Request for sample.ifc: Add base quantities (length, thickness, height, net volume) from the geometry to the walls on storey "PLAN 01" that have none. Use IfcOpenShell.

First a look at what the model holds.

```python
import ifcopenshell
import ifcopenshell.util.element
import ifcopenshell.util.unit

model = ifcopenshell.open("sample.ifc")
print(model.schema)
for unit_type in ("LENGTHUNIT", "AREAUNIT", "VOLUMEUNIT"):
    print(unit_type, ifcopenshell.util.unit.calculate_unit_scale(model, unit_type))
storey = next(s for s in model.by_type("IfcBuildingStorey") if s.Name == "PLAN 01")
walls = [e for e in ifcopenshell.util.element.get_decomposition(storey) if e.is_a("IfcWall")]
for e in sorted(walls, key=lambda e: e.id()):
    print(e.id(), e.is_a(), e.Name, list(ifcopenshell.util.element.get_psets(e, qtos_only=True)), sep=" | ")
```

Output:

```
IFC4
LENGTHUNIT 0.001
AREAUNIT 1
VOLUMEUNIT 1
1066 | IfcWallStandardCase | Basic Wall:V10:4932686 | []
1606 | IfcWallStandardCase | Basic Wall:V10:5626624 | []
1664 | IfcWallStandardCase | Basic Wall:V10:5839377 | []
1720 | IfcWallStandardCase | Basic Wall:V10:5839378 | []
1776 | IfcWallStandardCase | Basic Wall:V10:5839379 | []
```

```python
import ifcopenshell
import ifcopenshell.api.pset
import ifcopenshell.geom
import ifcopenshell.util.element
import ifcopenshell.util.shape
import ifcopenshell.util.unit

model = ifcopenshell.open("sample.ifc")
unit_scale = ifcopenshell.util.unit.calculate_unit_scale(model)
volume_scale = ifcopenshell.util.unit.calculate_unit_scale(model, "VOLUMEUNIT")
settings = ifcopenshell.geom.settings()

storey = next(s for s in model.by_type("IfcBuildingStorey") if s.Name == "PLAN 01")
walls = [e for e in ifcopenshell.util.element.get_decomposition(storey) if e.is_a("IfcWall")]

for e in sorted(walls, key=lambda e: e.id()):
    if ifcopenshell.util.element.get_psets(e, qtos_only=True, should_inherit=False):
        continue
    # Geometry comes back in metres, in the element's own axes.
    shape = ifcopenshell.geom.create_shape(settings, e)
    values = {
        "Length": ifcopenshell.util.shape.get_x(shape.geometry) / unit_scale,
        "Width": ifcopenshell.util.shape.get_y(shape.geometry) / unit_scale,
        "Height": ifcopenshell.util.shape.get_z(shape.geometry) / unit_scale,
        "NetVolume": ifcopenshell.util.shape.get_volume(shape.geometry) / volume_scale,
    }
    qto = ifcopenshell.api.pset.add_qto(model, product=e, name="Qto_WallBaseQuantities")
    ifcopenshell.api.pset.edit_qto(model, qto=qto, properties=values)
    print(e.id(), {k: round(v, 3) for k, v in values.items()})

model.write("sample_edited.ifc")
```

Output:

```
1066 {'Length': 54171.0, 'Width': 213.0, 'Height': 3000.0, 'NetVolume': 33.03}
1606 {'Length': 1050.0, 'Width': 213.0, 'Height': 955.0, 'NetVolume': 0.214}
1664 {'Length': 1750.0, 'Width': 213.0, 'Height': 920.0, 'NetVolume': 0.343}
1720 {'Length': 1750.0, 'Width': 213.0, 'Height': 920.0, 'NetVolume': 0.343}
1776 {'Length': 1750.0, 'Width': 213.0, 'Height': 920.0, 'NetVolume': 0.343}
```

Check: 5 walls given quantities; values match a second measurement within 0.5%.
